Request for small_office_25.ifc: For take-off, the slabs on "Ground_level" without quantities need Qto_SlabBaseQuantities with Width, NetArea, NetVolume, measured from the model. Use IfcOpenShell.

First a look at what the model holds.

```python
import ifcopenshell
import ifcopenshell.util.element
import ifcopenshell.util.unit

model = ifcopenshell.open("small_office_25.ifc")
print(model.schema)
for unit_type in ("LENGTHUNIT", "AREAUNIT", "VOLUMEUNIT"):
    print(unit_type, ifcopenshell.util.unit.calculate_unit_scale(model, unit_type))
storey = next(s for s in model.by_type("IfcBuildingStorey") if s.Name == "Ground_level")
slabs = [e for e in ifcopenshell.util.element.get_decomposition(storey) if e.is_a("IfcSlab")]
for e in sorted(slabs, key=lambda e: e.id()):
    print(e.id(), e.is_a(), e.Name, list(ifcopenshell.util.element.get_psets(e, qtos_only=True)), sep=" | ")
```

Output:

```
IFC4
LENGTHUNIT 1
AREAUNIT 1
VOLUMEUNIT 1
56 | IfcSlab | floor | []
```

```python
import ifcopenshell
import ifcopenshell.api.pset
import ifcopenshell.geom
import ifcopenshell.util.element
import ifcopenshell.util.shape
import ifcopenshell.util.unit

model = ifcopenshell.open("small_office_25.ifc")
unit_scale = ifcopenshell.util.unit.calculate_unit_scale(model)
area_scale = ifcopenshell.util.unit.calculate_unit_scale(model, "AREAUNIT")
volume_scale = ifcopenshell.util.unit.calculate_unit_scale(model, "VOLUMEUNIT")
settings = ifcopenshell.geom.settings()

storey = next(s for s in model.by_type("IfcBuildingStorey") if s.Name == "Ground_level")
slabs = [e for e in ifcopenshell.util.element.get_decomposition(storey) if e.is_a("IfcSlab")]

for e in sorted(slabs, key=lambda e: e.id()):
    if ifcopenshell.util.element.get_psets(e, qtos_only=True, should_inherit=False):
        continue
    # Geometry comes back in metres, in the element's own axes.
    shape = ifcopenshell.geom.create_shape(settings, e)
    values = {
        "Width": ifcopenshell.util.shape.get_z(shape.geometry) / unit_scale,
        "NetArea": ifcopenshell.util.shape.get_footprint_area(shape.geometry) / area_scale,
        "NetVolume": ifcopenshell.util.shape.get_volume(shape.geometry) / volume_scale,
    }
    qto = ifcopenshell.api.pset.add_qto(model, product=e, name="Qto_SlabBaseQuantities")
    ifcopenshell.api.pset.edit_qto(model, qto=qto, properties=values)
    print(e.id(), {k: round(v, 3) for k, v in values.items()})

model.write("small_office_25_updated.ifc")
```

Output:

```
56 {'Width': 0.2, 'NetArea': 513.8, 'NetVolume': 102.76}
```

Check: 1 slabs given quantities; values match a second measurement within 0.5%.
